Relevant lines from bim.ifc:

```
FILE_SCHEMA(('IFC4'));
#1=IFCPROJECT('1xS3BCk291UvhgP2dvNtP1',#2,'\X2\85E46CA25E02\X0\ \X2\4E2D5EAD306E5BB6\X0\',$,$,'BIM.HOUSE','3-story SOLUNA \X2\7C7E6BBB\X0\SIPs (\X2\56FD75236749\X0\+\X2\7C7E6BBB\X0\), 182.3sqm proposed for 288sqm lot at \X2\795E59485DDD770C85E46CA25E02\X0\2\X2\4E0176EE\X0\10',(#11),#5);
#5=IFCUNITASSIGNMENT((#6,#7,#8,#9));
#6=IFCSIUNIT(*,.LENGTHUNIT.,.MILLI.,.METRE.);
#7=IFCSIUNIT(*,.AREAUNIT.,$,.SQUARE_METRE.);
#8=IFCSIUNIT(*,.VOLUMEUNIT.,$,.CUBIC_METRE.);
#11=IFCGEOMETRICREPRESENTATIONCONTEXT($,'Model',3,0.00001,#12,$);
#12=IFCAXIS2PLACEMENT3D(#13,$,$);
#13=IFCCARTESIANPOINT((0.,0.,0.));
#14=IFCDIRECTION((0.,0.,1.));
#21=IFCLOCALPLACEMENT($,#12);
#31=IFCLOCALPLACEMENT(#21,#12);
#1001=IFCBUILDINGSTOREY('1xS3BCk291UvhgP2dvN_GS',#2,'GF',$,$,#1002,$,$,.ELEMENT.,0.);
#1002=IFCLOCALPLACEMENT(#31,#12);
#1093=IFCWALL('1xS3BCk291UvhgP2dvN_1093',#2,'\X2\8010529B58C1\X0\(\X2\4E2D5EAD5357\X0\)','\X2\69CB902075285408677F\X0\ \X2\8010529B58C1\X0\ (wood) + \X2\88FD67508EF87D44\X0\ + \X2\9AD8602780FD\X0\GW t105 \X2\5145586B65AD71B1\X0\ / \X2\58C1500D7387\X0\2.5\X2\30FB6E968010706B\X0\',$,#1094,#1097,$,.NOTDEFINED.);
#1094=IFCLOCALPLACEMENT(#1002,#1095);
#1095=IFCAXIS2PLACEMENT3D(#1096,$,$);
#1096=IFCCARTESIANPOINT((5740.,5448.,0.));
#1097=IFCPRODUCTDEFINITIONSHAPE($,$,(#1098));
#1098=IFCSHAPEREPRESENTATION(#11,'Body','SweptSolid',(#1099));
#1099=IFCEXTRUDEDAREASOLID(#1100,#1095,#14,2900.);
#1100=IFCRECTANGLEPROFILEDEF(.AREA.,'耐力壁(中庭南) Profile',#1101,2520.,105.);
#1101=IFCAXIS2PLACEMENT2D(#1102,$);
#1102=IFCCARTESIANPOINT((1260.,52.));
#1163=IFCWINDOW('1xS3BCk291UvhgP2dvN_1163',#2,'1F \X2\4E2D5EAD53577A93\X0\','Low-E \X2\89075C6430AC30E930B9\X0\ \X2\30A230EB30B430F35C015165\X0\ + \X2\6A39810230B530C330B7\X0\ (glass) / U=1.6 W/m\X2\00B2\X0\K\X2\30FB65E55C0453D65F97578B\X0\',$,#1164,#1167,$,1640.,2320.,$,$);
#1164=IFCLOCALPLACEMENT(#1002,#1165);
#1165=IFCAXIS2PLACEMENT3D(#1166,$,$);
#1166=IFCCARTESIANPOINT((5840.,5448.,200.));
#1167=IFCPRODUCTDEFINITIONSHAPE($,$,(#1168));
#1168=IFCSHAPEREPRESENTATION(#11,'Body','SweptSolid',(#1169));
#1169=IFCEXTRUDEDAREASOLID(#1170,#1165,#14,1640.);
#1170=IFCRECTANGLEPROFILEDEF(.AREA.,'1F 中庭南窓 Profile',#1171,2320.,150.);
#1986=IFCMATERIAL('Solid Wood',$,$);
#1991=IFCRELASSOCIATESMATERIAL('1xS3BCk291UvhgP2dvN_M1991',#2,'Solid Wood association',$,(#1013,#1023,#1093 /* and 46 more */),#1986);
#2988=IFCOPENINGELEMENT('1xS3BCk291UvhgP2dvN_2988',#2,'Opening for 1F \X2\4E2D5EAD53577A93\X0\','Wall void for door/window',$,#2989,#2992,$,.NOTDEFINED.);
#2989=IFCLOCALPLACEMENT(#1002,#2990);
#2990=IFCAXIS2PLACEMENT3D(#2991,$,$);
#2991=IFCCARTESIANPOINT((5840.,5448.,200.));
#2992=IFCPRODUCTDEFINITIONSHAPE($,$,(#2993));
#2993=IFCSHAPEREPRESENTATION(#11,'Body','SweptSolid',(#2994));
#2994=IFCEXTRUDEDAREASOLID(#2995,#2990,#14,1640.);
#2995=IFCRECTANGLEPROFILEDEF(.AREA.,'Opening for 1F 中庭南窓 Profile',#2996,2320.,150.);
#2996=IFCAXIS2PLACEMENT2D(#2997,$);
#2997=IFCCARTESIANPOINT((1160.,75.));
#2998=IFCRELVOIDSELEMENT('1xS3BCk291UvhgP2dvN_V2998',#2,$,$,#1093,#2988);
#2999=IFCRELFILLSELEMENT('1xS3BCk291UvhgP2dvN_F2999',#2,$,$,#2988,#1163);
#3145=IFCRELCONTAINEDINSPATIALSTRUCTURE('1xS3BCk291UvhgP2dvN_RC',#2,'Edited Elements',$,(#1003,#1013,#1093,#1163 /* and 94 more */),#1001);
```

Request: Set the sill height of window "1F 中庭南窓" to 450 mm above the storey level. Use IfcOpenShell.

```python
import numpy as np
import ifcopenshell
import ifcopenshell.api.geometry
import ifcopenshell.geom
import ifcopenshell.util.element
import ifcopenshell.util.placement
import ifcopenshell.util.shape
import ifcopenshell.util.unit

model = ifcopenshell.open("bim.ifc")
unit_scale = ifcopenshell.util.unit.calculate_unit_scale(model)

window = model.by_guid("1xS3BCk291UvhgP2dvN_1163")
opening = window.FillsVoids[0].RelatingOpeningElement
storey = ifcopenshell.util.element.get_container(window, ifc_class="IfcBuildingStorey")
level = ifcopenshell.util.placement.get_local_placement(storey.ObjectPlacement)[2, 3]

# The opening's origin need not be at the sill, so measure its lowest point.
shape = ifcopenshell.geom.create_shape(ifcopenshell.geom.settings(), opening)
bottom = ifcopenshell.util.shape.get_shape_bottom_elevation(shape, shape.geometry) / unit_scale
dz = level + 0.45 / unit_scale - bottom

shift = np.array([0.0, 0.0, dz])
# The window is not placed relative to its opening, so move both.
for product in (opening, window):
    matrix = ifcopenshell.util.placement.get_local_placement(product.ObjectPlacement)
    matrix[:3, 3] += shift
    ifcopenshell.api.geometry.edit_object_placement(model, product=product, matrix=matrix, is_si=False)

print(f"moved by {dz * unit_scale:+.3f} m")

model.write("bim_edited.ifc")
```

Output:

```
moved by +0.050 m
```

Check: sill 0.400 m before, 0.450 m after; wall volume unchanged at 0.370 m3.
